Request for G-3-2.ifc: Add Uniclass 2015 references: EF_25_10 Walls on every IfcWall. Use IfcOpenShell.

First a look at what the model holds.

```python
import ifcopenshell

model = ifcopenshell.open("G-3-2.ifc")
print(model.schema)
print("classifications:", [c.Name for c in model.by_type("IfcClassification")])
for ifc_class in ("IfcDoor", "IfcRoof", "IfcStair", "IfcWall", "IfcWindow"):
    print(ifc_class, len(model.by_type(ifc_class)))
```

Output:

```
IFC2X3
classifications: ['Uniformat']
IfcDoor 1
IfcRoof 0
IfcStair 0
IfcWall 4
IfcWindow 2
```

```python
import ifcopenshell
import ifcopenshell.api.classification

model = ifcopenshell.open("G-3-2.ifc")

# IFC2X3 requires Source and Edition and has no link from the project to the system.
system = model.create_entity("IfcClassification", Source="NBS", Edition="2015", Name="Uniclass 2015")

codes = {
    "IfcWall": ("EF_25_10", "Walls"),
}
for ifc_class, (code, name) in codes.items():
    products = model.by_type(ifc_class)
    ifcopenshell.api.classification.add_reference(
        model, products=products, classification=system, identification=code, name=name
    )
    print(code, len(products))

model.write("G-3-2-out.ifc")
```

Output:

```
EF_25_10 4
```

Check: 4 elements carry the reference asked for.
